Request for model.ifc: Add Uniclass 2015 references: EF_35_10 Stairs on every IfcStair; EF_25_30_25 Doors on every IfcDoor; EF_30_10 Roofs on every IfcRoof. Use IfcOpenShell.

First a look at what the model holds.

```python
import ifcopenshell

model = ifcopenshell.open("model.ifc")
print(model.schema)
print("classifications:", [c.Name for c in model.by_type("IfcClassification")])
for ifc_class in ("IfcDoor", "IfcRoof", "IfcStair", "IfcWall", "IfcWindow"):
    print(ifc_class, len(model.by_type(ifc_class)))
```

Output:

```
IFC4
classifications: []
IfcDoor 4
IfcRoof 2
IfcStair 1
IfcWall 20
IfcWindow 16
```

```python
import ifcopenshell
import ifcopenshell.api.classification

model = ifcopenshell.open("model.ifc")

system = ifcopenshell.api.classification.add_classification(model, classification="Uniclass 2015")

codes = {
    "IfcStair": ("EF_35_10", "Stairs"),
    "IfcDoor": ("EF_25_30_25", "Doors"),
    "IfcRoof": ("EF_30_10", "Roofs"),
}
for ifc_class, (code, name) in codes.items():
    products = model.by_type(ifc_class)
    ifcopenshell.api.classification.add_reference(
        model, products=products, classification=system, identification=code, name=name
    )
    print(code, len(products))

model.write("model_updated.ifc")
```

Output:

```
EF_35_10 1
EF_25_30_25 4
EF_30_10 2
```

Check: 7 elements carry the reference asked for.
